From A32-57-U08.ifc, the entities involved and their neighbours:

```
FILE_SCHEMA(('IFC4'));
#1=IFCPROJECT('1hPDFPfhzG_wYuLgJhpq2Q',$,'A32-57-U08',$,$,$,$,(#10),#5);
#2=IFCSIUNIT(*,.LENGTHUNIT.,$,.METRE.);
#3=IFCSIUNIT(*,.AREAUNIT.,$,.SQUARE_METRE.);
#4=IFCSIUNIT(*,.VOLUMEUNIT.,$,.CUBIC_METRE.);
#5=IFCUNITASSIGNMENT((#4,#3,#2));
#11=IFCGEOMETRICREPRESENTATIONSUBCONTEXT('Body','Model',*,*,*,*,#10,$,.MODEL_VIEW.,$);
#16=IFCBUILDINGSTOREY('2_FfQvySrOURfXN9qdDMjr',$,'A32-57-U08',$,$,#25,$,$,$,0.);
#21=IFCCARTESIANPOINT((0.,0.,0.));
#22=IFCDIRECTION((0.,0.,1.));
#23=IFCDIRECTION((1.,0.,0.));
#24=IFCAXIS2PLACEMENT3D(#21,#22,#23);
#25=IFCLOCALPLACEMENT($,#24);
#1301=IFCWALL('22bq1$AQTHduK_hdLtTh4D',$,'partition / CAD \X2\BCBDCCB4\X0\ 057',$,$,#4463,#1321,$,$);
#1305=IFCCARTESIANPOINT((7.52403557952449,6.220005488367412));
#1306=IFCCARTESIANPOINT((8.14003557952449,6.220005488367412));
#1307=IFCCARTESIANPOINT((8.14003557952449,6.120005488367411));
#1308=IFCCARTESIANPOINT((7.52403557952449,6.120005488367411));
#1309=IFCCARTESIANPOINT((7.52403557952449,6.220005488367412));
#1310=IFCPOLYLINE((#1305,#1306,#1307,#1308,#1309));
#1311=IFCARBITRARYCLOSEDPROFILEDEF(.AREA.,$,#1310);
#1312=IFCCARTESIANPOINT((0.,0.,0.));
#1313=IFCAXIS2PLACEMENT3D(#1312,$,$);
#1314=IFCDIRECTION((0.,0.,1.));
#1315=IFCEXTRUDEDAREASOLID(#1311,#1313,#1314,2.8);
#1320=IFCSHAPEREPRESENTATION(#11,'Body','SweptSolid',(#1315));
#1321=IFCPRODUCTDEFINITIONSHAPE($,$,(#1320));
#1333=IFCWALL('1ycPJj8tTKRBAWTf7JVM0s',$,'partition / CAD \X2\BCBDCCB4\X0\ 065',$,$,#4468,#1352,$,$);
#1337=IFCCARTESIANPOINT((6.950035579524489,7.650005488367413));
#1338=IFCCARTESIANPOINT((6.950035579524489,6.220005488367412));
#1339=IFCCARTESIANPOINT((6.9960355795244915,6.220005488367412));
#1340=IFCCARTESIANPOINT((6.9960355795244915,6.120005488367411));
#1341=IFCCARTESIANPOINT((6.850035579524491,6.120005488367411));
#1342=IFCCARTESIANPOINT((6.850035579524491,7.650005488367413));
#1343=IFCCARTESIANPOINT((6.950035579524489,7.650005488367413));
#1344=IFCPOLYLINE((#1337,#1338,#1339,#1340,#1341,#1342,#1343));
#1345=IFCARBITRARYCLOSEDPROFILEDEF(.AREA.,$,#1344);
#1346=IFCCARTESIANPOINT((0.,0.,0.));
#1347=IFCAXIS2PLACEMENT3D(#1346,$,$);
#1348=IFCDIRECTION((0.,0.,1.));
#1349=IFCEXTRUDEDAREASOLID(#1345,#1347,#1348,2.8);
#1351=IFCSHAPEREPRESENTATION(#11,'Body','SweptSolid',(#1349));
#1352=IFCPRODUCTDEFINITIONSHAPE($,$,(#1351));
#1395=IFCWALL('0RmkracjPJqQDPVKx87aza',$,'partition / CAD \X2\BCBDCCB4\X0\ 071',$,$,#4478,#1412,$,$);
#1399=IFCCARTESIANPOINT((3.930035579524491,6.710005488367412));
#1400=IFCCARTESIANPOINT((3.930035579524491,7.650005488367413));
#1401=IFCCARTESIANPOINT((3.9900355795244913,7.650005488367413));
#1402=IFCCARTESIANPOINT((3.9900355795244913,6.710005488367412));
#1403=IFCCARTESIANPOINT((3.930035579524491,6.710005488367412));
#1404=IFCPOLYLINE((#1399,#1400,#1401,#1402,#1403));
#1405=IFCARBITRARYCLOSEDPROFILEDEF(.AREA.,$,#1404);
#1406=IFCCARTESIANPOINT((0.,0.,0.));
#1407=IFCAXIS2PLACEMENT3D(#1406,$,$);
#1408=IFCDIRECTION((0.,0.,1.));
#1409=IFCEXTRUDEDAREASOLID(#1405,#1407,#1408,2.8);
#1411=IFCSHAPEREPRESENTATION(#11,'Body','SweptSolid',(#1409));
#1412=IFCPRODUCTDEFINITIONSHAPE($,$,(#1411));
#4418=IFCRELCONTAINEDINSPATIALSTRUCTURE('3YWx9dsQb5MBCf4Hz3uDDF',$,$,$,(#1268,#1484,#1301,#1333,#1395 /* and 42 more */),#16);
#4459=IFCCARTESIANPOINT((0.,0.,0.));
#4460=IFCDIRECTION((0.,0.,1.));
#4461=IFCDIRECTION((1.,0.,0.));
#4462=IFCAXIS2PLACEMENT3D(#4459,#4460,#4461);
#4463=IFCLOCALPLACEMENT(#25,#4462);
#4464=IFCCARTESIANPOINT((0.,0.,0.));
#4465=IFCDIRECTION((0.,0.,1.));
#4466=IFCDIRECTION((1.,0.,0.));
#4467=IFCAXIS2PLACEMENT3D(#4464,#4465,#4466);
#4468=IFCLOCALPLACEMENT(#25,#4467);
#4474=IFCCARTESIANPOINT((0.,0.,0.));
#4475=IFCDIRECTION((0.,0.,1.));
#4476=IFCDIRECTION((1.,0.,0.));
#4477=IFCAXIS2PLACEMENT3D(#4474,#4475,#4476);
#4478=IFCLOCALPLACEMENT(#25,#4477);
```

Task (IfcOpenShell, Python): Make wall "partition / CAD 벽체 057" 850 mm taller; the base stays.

```python
import ifcopenshell
import ifcopenshell.geom
import ifcopenshell.util.representation
import ifcopenshell.util.shape

model = ifcopenshell.open("A32-57-U08.ifc")
settings = ifcopenshell.geom.settings()


def volume(element):
    """Net volume in cubic metres, openings subtracted."""
    shape = ifcopenshell.geom.create_shape(settings, element)
    return ifcopenshell.util.shape.get_volume(shape.geometry)


wall = model.by_guid("22bq1$AQTHduK_hdLtTh4D")
before = volume(wall)

body = ifcopenshell.util.representation.get_representation(wall, "Model", "Body")
solid = body.Items[0]
old_height = solid.Depth
solid.Depth += 0.85
after = volume(wall)

print(f"height {old_height:g} -> {solid.Depth:g}, volume {before:.3f} -> {after:.3f} m3")

model.write("A32-57-U08_updated.ifc")
```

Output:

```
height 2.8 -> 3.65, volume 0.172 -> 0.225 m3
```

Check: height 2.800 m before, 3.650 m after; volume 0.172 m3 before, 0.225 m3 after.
